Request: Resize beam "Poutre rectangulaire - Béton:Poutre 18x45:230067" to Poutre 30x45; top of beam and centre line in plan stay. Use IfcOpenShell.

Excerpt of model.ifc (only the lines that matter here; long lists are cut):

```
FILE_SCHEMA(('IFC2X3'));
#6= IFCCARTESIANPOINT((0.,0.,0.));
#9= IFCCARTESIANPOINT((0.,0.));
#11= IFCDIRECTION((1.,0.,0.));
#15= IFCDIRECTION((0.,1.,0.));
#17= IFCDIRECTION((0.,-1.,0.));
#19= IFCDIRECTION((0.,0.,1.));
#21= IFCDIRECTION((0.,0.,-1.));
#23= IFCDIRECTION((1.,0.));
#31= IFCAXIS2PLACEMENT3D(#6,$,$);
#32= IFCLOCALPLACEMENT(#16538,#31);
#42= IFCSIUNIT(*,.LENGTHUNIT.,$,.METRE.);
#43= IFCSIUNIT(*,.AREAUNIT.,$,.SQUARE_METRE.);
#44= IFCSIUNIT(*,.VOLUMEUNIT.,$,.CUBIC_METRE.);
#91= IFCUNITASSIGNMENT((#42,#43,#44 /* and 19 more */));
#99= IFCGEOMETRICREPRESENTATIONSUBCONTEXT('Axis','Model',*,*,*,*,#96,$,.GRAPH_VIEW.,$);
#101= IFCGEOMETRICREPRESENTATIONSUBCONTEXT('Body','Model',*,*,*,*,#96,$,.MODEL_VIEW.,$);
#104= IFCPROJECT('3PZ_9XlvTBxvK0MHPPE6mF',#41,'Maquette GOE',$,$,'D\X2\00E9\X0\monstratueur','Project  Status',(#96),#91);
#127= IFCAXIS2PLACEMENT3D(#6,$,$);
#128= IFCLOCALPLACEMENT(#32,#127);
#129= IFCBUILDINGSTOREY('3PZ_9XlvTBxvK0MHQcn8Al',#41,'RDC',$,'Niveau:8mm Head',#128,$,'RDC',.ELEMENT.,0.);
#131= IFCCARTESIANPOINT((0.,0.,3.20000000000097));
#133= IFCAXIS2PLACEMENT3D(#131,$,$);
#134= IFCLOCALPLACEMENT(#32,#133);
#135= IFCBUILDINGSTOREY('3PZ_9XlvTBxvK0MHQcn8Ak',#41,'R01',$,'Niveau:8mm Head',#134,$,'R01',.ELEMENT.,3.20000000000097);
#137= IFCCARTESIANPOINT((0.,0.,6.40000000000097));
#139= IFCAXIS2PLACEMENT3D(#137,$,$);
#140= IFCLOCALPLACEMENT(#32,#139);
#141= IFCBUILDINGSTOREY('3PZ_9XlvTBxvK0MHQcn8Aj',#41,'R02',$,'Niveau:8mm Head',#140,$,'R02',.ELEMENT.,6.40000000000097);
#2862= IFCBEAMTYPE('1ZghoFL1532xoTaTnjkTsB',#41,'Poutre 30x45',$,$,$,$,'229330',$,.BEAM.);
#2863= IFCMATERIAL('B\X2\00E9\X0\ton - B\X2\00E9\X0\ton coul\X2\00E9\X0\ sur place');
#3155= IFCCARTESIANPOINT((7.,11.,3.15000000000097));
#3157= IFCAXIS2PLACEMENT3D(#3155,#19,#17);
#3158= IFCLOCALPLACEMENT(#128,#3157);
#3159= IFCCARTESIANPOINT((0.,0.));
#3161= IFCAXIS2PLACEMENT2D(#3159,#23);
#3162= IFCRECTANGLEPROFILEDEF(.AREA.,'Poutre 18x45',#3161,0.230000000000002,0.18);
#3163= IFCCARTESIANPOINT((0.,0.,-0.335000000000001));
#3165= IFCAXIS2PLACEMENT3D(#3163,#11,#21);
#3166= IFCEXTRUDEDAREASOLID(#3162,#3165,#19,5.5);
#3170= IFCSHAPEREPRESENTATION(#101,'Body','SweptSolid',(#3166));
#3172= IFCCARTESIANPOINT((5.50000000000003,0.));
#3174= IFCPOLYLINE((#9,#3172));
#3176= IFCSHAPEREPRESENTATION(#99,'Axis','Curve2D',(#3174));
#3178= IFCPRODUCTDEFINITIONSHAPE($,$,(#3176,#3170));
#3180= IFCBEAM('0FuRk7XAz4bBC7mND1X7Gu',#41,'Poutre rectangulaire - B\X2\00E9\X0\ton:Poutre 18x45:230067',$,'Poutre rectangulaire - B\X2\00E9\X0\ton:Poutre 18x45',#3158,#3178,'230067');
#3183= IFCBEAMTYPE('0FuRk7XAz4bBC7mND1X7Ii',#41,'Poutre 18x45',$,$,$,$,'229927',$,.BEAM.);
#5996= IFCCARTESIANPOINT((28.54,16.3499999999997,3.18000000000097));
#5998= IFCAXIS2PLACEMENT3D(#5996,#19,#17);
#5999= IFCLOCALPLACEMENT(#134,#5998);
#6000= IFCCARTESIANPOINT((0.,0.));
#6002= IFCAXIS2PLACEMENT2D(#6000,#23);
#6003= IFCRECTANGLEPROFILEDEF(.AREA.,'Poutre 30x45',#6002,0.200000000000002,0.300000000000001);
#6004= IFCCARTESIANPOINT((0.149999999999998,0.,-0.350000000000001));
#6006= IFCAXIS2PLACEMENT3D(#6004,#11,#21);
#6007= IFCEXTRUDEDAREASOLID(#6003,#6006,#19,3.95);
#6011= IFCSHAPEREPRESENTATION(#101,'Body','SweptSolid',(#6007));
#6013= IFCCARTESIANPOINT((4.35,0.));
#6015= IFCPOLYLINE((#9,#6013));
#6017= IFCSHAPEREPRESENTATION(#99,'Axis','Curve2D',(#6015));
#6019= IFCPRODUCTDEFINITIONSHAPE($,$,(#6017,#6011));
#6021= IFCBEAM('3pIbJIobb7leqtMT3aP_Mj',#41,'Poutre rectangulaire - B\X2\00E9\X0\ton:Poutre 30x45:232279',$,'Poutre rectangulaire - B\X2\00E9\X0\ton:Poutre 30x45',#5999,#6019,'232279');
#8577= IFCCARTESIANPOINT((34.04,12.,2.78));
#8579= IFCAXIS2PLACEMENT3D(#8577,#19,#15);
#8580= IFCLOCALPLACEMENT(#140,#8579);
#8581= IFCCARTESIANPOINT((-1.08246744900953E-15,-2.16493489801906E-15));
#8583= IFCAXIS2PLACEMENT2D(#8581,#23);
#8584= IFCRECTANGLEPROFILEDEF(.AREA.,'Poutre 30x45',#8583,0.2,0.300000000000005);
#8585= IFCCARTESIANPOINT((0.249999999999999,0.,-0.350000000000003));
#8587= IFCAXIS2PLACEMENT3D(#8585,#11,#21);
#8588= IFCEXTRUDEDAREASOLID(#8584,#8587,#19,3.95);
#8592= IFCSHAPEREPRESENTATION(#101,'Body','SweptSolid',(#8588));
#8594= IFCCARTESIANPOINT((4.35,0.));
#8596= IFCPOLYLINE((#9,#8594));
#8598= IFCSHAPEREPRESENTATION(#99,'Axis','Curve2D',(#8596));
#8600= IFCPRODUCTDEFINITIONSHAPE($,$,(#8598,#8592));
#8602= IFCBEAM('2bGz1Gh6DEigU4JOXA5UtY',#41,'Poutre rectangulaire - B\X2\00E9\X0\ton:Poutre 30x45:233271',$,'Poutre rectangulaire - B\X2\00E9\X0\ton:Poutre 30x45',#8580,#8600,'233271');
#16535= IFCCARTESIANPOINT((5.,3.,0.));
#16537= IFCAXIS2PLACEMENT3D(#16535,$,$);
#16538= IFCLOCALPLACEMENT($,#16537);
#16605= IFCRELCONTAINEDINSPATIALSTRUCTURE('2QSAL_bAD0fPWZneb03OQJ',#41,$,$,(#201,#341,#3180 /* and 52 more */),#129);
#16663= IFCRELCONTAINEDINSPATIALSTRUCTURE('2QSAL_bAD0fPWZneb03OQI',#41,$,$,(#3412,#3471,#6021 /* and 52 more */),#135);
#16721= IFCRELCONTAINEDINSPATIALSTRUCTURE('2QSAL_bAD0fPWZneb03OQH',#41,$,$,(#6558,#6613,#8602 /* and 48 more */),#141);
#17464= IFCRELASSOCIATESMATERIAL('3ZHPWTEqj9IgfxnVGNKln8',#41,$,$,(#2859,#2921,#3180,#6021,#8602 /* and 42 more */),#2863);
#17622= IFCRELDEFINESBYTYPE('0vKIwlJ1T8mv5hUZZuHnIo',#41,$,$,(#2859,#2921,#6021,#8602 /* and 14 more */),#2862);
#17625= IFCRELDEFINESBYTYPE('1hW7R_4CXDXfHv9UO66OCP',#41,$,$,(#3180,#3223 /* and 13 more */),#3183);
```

```python
import ifcopenshell
import ifcopenshell.api.type
import ifcopenshell.util.element
import ifcopenshell.util.representation

model = ifcopenshell.open("model.ifc")

member = model.by_guid("0FuRk7XAz4bBC7mND1X7Gu")
source = next(p for p in model.by_type("IfcRectangleProfileDef") if p.ProfileName == "Poutre 30x45")

body = ifcopenshell.util.representation.get_representation(member, "Model", "Body")
solid = body.Items[0]
old_profile = solid.SweptArea

# Copy the section's sizes but keep this member's own profile position.
profile = ifcopenshell.util.element.copy(model, source)
# Profiles are centred, so shift by half the change in depth to hold the top.
shift = (old_profile.XDim - profile.XDim) / 2
x, y = old_profile.Position.Location.Coordinates
up = (-1.0, 0.0)  # upwards, in the solid's own plane
location = model.createIfcCartesianPoint((x + up[0] * shift, y + up[1] * shift))
profile.Position = model.createIfcAxis2Placement2D(location, old_profile.Position.RefDirection)
solid.SweptArea = profile
if not model.get_total_inverses(old_profile):
    ifcopenshell.util.element.remove_deep2(model, old_profile)

new_type = model.by_guid("1ZghoFL1532xoTaTnjkTsB")
ifcopenshell.api.type.assign_type(
    model, related_objects=[member], relating_type=new_type, should_map_representations=False
)
member.Name = member.Name.replace("Poutre 18x45", "Poutre 30x45")
member.ObjectType = "Poutre rectangulaire - Béton:Poutre 30x45"

print(solid.SweptArea)

model.write("model_v2.ifc")
```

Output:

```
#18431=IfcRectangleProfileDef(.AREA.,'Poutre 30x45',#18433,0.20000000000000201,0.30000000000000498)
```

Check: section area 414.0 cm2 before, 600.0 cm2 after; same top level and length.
